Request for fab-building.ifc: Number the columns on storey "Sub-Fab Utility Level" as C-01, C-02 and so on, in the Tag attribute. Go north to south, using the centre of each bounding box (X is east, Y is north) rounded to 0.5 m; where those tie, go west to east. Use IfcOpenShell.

First a look at what the model holds.

```python
import ifcopenshell
import ifcopenshell.util.element
import ifcopenshell.util.placement

model = ifcopenshell.open("fab-building.ifc")
print(model.schema)
storey = next(s for s in model.by_type("IfcBuildingStorey") if s.Name == "Sub-Fab Utility Level")
columns = [e for e in ifcopenshell.util.element.get_decomposition(storey) if e.is_a("IfcColumn")]
for e in sorted(columns, key=lambda e: e.id()):
    origin = ifcopenshell.util.placement.get_local_placement(e.ObjectPlacement)[:3, 3]
    print(e.id(), e.Tag, e.Name, origin.round(2) + 0.0, sep=" | ")
```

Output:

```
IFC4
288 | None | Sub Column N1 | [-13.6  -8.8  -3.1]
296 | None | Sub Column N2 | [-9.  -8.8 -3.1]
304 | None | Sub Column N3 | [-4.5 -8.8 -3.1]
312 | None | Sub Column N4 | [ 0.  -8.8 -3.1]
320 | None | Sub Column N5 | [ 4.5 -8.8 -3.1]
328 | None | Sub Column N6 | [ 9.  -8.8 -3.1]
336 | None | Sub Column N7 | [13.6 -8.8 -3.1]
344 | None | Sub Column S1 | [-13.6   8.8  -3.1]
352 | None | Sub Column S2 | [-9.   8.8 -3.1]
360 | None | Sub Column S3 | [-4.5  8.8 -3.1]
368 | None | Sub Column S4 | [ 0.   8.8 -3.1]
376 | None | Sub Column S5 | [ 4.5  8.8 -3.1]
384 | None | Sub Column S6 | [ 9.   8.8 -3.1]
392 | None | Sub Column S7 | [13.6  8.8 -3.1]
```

```python
import ifcopenshell
import ifcopenshell.geom
import ifcopenshell.util.element
import ifcopenshell.util.shape

model = ifcopenshell.open("fab-building.ifc")
settings = ifcopenshell.geom.settings()
settings.set("use-world-coords", True)


def centre(element):
    shape = ifcopenshell.geom.create_shape(settings, element)
    return ifcopenshell.util.shape.get_bbox_centroid(shape.geometry)


storey = next(s for s in model.by_type("IfcBuildingStorey") if s.Name == "Sub-Fab Utility Level")
columns = [e for e in ifcopenshell.util.element.get_decomposition(storey) if e.is_a("IfcColumn")]

# Insertion points can sit at a corner or the storey origin, so sort by the geometry (in metres).
centres = {e: centre(e) for e in columns}
columns.sort(key=lambda e: (-round(centres[e][1] / 0.5), centres[e][0]))

for i, e in enumerate(columns, start=1):
    number = f"C-{i:02d}"
    e.Tag = number
    print(e.id(), number)

model.write("fab-building-out.ifc")
```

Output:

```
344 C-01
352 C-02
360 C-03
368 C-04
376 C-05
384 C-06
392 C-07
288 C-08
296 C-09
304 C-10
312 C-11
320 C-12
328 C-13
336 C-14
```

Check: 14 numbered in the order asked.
